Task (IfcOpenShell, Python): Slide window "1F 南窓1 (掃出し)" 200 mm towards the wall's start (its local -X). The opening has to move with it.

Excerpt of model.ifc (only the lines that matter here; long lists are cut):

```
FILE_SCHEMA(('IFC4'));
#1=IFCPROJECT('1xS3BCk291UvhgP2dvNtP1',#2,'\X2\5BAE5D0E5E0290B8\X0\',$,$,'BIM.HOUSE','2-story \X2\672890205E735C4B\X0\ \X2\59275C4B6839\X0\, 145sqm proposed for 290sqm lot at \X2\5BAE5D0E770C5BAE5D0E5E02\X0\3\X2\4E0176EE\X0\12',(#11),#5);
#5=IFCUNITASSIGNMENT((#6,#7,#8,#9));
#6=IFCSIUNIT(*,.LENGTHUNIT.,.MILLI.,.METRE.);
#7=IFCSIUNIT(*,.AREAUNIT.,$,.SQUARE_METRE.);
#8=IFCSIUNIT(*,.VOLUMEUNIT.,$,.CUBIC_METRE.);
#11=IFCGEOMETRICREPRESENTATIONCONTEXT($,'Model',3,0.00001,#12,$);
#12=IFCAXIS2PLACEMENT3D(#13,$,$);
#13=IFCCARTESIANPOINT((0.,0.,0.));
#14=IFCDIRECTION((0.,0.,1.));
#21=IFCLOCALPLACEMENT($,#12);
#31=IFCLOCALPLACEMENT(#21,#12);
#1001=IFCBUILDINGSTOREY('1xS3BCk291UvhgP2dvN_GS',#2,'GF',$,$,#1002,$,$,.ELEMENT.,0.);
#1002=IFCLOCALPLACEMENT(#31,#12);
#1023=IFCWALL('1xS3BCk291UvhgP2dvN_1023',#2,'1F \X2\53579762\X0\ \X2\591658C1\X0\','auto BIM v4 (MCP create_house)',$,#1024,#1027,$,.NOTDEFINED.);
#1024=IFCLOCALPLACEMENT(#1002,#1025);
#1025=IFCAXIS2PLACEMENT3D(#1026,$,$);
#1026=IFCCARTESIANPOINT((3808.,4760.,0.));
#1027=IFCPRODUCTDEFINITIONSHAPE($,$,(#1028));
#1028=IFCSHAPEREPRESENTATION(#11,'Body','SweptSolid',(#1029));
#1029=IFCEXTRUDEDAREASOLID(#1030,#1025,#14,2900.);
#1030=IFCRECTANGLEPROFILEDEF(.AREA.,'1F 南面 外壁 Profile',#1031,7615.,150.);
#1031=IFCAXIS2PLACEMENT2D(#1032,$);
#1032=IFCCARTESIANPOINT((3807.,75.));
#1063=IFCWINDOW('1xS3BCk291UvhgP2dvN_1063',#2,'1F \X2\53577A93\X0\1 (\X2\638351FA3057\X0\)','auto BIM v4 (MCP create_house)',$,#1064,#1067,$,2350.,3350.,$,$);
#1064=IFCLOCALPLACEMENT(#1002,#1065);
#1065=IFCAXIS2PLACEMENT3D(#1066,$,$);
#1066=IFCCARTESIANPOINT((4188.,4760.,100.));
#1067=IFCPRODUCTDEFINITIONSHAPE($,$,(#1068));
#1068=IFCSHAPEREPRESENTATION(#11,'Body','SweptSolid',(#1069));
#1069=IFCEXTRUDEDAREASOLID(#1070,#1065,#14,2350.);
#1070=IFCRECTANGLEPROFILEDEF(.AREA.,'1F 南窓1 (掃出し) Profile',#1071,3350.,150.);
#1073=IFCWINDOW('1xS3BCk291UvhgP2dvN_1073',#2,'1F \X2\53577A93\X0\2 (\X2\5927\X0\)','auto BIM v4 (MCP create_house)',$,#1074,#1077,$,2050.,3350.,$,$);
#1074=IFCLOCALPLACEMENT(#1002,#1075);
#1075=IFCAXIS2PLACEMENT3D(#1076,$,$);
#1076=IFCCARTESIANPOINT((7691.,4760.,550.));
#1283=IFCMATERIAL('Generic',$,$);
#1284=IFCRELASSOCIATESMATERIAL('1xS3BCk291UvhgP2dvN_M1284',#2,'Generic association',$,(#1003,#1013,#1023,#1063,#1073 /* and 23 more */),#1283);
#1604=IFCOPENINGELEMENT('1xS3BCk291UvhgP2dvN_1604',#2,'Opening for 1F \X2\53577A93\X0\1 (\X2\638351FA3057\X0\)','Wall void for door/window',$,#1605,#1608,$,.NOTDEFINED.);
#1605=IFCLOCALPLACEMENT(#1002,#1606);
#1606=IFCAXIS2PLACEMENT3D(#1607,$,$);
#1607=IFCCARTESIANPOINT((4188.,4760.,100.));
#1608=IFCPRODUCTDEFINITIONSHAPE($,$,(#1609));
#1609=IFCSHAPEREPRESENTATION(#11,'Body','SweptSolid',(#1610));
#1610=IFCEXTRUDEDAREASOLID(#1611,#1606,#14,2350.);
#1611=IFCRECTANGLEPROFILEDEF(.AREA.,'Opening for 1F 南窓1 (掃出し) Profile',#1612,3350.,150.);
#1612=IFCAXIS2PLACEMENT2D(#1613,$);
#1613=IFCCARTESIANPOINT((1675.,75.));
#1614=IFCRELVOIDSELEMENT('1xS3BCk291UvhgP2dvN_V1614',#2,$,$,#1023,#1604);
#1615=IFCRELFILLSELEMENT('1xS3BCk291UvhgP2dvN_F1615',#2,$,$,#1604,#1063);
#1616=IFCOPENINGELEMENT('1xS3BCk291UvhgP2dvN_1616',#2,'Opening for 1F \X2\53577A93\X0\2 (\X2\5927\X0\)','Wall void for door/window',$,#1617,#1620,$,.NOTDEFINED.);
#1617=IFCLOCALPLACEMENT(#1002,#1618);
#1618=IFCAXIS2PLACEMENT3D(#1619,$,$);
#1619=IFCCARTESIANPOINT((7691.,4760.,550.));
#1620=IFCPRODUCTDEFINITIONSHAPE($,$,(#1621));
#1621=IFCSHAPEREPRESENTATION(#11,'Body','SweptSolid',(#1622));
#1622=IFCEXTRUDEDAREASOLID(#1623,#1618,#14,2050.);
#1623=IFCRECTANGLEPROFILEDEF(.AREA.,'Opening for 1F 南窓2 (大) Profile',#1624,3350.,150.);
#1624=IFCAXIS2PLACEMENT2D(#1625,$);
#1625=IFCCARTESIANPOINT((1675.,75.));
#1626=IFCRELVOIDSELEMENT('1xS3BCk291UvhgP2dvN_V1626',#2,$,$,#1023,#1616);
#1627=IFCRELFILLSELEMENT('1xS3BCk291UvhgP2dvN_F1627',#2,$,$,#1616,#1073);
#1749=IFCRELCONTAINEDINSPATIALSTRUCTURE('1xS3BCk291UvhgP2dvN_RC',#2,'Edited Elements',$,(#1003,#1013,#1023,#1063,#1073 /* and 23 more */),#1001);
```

```python
import ifcopenshell
import ifcopenshell.api.geometry
import ifcopenshell.util.placement
import ifcopenshell.util.unit

model = ifcopenshell.open("model.ifc")
unit_scale = ifcopenshell.util.unit.calculate_unit_scale(model)

window = model.by_id(1063)
opening = window.FillsVoids[0].RelatingOpeningElement
wall = opening.VoidsElements[0].RelatingBuildingElement

wall_matrix = ifcopenshell.util.placement.get_local_placement(wall.ObjectPlacement)
shift = wall_matrix[:3, 0] * -0.2 / unit_scale
before = ifcopenshell.util.placement.get_local_placement(window.ObjectPlacement)[:3, 3].copy()

# The window is not placed relative to its opening, so move both.
for product in (opening, window):
    matrix = ifcopenshell.util.placement.get_local_placement(product.ObjectPlacement)
    matrix[:3, 3] += shift
    ifcopenshell.api.geometry.edit_object_placement(model, product=product, matrix=matrix, is_si=False)

after = ifcopenshell.util.placement.get_local_placement(window.ObjectPlacement)[:3, 3]
print("window moved by", (after - before).round(3) + 0.0)

model.write("model_edited.ifc")
```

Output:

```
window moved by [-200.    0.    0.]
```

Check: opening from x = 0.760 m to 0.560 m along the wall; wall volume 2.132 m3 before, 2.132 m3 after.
